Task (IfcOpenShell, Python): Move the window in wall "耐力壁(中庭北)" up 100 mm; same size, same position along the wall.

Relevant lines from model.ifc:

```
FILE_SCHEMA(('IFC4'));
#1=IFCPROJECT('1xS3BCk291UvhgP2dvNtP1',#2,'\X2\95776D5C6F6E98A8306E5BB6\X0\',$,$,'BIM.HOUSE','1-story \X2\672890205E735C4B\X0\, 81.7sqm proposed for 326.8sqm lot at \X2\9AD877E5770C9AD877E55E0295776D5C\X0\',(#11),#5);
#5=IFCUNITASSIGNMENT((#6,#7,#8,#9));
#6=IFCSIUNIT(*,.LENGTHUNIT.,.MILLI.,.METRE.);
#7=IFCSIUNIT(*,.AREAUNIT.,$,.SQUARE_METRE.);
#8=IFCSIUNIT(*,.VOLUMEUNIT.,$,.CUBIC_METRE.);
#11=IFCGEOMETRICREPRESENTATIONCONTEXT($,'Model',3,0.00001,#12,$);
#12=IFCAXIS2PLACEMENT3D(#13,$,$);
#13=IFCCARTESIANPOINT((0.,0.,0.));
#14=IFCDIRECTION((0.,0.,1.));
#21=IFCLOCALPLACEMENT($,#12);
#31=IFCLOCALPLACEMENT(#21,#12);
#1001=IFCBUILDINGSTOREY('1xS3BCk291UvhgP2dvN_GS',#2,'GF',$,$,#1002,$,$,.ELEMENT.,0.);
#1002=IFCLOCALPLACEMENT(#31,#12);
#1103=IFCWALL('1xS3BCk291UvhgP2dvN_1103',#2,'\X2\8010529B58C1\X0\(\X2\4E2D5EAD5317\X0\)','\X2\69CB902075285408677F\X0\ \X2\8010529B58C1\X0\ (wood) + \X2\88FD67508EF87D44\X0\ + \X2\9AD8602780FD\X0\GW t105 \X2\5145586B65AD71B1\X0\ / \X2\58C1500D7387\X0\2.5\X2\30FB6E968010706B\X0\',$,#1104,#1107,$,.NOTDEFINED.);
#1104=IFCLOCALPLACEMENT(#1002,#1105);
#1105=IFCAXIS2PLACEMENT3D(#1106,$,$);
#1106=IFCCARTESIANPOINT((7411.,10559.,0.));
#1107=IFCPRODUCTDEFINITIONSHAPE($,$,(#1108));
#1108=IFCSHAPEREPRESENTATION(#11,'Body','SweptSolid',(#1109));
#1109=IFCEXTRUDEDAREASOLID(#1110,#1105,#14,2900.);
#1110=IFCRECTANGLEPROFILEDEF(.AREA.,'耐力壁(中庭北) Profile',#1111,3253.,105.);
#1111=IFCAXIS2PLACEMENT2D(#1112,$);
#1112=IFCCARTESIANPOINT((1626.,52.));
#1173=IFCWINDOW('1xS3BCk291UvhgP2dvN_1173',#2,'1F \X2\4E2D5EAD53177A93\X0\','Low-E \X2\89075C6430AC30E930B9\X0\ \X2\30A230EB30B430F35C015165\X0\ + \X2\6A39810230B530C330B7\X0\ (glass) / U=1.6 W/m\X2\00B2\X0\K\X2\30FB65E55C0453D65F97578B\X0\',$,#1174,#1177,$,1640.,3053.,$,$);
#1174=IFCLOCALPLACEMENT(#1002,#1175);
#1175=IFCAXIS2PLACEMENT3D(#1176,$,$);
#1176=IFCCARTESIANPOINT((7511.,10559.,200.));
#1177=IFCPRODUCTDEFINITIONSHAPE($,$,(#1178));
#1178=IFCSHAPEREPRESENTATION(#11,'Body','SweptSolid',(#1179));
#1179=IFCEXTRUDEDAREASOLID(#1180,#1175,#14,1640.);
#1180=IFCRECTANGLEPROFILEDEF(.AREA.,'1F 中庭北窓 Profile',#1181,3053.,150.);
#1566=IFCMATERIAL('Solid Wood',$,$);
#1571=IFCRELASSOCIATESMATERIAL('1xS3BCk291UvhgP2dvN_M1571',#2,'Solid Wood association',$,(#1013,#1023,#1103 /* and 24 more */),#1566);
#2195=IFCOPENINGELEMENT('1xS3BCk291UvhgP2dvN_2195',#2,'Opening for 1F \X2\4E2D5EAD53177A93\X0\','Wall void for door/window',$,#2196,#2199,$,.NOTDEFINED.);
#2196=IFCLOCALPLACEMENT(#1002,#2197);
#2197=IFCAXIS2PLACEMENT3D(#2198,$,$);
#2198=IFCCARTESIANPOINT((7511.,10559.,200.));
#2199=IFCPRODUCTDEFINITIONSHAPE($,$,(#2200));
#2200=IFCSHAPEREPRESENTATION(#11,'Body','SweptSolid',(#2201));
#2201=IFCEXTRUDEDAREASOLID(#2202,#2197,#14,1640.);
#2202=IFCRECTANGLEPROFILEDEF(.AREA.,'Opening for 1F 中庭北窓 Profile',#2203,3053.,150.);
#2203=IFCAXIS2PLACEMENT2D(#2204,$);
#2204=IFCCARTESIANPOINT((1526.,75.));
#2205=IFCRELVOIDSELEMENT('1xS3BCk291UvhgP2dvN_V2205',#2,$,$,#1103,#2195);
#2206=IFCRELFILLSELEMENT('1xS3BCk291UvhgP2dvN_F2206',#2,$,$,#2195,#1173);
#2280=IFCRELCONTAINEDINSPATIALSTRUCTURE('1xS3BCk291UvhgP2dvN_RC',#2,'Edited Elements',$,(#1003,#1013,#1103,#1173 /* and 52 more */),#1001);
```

```python
import numpy as np
import ifcopenshell
import ifcopenshell.api.geometry
import ifcopenshell.util.placement
import ifcopenshell.util.unit

model = ifcopenshell.open("model.ifc")
unit_scale = ifcopenshell.util.unit.calculate_unit_scale(model)

window = model.by_guid("1xS3BCk291UvhgP2dvN_1173")
opening = window.FillsVoids[0].RelatingOpeningElement
dz = 0.1 / unit_scale

shift = np.array([0.0, 0.0, dz])
# The window is not placed relative to its opening, so move both.
for product in (opening, window):
    matrix = ifcopenshell.util.placement.get_local_placement(product.ObjectPlacement)
    matrix[:3, 3] += shift
    ifcopenshell.api.geometry.edit_object_placement(model, product=product, matrix=matrix, is_si=False)

print(f"moved by {dz * unit_scale:+.3f} m")

model.write("model_rev.ifc")
```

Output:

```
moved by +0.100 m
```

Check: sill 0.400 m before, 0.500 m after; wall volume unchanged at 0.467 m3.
